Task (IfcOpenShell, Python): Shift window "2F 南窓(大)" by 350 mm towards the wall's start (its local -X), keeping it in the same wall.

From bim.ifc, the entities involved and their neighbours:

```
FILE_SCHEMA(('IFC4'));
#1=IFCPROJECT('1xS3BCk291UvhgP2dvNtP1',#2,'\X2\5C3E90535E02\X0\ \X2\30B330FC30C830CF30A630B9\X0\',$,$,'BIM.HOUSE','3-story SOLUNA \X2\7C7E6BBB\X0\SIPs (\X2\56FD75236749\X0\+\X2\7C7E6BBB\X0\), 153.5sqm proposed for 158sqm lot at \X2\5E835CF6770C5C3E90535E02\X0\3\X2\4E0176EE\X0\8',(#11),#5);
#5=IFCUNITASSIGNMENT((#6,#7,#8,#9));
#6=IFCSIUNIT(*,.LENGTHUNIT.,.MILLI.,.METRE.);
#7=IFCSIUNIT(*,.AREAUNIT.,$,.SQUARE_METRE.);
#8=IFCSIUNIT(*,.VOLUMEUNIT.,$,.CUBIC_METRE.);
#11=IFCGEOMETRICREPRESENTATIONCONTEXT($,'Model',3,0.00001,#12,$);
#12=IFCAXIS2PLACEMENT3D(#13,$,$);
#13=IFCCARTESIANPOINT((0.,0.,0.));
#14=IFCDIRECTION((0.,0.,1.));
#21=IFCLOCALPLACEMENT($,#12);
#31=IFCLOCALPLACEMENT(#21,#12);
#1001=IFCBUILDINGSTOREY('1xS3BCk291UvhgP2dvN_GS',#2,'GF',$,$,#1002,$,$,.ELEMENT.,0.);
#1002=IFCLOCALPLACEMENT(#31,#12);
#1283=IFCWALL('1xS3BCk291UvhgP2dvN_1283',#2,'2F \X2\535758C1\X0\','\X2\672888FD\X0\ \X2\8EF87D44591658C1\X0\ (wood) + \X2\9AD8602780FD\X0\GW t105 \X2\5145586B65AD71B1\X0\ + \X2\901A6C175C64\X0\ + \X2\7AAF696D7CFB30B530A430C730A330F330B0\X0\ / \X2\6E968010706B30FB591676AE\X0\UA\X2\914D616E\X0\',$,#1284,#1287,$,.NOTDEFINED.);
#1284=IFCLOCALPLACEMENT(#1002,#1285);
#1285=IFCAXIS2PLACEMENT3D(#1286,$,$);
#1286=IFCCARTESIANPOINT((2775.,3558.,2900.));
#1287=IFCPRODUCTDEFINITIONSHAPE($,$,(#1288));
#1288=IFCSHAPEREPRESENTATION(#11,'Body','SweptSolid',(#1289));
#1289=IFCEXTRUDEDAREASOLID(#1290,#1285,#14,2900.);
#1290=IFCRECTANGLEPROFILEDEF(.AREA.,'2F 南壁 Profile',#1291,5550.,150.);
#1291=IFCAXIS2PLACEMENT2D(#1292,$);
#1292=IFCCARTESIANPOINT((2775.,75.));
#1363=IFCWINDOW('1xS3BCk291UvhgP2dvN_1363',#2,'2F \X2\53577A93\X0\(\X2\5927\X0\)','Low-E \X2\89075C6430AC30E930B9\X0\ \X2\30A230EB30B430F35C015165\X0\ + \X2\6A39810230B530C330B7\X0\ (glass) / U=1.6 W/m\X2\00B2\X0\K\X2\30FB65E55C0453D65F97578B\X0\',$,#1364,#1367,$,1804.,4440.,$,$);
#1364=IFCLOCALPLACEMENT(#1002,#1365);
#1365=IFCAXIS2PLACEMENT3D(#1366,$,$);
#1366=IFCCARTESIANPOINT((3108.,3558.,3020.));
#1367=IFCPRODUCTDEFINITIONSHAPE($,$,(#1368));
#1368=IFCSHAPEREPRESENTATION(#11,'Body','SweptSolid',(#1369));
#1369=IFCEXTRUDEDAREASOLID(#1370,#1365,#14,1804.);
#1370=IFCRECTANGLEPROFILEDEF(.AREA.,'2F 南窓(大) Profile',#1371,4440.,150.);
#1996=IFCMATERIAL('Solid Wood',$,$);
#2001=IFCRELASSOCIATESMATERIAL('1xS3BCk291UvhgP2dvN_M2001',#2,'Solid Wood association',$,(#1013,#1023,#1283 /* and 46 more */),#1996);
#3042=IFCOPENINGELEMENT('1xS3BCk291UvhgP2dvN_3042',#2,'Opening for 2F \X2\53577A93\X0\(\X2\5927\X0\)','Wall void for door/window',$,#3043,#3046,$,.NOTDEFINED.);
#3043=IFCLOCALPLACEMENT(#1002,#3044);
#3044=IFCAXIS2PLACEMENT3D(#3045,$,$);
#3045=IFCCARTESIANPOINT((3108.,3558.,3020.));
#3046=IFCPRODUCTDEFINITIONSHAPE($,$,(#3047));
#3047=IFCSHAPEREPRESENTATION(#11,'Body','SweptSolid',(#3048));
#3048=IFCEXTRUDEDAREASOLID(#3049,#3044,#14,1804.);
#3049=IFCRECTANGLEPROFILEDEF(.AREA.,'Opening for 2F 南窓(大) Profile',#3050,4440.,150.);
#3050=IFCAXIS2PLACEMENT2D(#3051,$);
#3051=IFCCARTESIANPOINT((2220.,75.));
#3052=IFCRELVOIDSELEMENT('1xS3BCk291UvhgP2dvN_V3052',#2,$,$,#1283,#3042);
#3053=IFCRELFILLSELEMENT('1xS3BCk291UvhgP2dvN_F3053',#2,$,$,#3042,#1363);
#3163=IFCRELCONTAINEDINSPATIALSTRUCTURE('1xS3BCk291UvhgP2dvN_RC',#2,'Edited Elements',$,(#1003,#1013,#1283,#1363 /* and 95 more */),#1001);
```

```python
import ifcopenshell
import ifcopenshell.api.geometry
import ifcopenshell.util.placement
import ifcopenshell.util.unit

model = ifcopenshell.open("bim.ifc")
unit_scale = ifcopenshell.util.unit.calculate_unit_scale(model)

window = model.by_guid("1xS3BCk291UvhgP2dvN_1363")
opening = window.FillsVoids[0].RelatingOpeningElement
wall = opening.VoidsElements[0].RelatingBuildingElement

wall_matrix = ifcopenshell.util.placement.get_local_placement(wall.ObjectPlacement)
shift = wall_matrix[:3, 0] * -0.35 / unit_scale
before = ifcopenshell.util.placement.get_local_placement(window.ObjectPlacement)[:3, 3].copy()

# The window is not placed relative to its opening, so move both.
for product in (opening, window):
    matrix = ifcopenshell.util.placement.get_local_placement(product.ObjectPlacement)
    matrix[:3, 3] += shift
    ifcopenshell.api.geometry.edit_object_placement(model, product=product, matrix=matrix, is_si=False)

after = ifcopenshell.util.placement.get_local_placement(window.ObjectPlacement)[:3, 3]
print("window moved by", (after - before).round(3) + 0.0)

model.write("bim-out.ifc")
```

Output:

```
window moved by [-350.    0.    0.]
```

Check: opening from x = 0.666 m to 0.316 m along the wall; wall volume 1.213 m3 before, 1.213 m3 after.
